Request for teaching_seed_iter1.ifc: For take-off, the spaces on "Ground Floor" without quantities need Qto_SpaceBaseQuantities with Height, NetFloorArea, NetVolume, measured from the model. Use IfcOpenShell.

First a look at what the model holds.

```python
import ifcopenshell
import ifcopenshell.util.element
import ifcopenshell.util.unit

model = ifcopenshell.open("teaching_seed_iter1.ifc")
print(model.schema)
for unit_type in ("LENGTHUNIT", "AREAUNIT", "VOLUMEUNIT"):
    print(unit_type, ifcopenshell.util.unit.calculate_unit_scale(model, unit_type))
storey = next(s for s in model.by_type("IfcBuildingStorey") if s.Name == "Ground Floor")
spaces = [e for e in ifcopenshell.util.element.get_decomposition(storey) if e.is_a("IfcSpace")]
for e in sorted(spaces, key=lambda e: e.id()):
    print(e.id(), e.is_a(), e.Name, list(ifcopenshell.util.element.get_psets(e, qtos_only=True)), sep=" | ")
```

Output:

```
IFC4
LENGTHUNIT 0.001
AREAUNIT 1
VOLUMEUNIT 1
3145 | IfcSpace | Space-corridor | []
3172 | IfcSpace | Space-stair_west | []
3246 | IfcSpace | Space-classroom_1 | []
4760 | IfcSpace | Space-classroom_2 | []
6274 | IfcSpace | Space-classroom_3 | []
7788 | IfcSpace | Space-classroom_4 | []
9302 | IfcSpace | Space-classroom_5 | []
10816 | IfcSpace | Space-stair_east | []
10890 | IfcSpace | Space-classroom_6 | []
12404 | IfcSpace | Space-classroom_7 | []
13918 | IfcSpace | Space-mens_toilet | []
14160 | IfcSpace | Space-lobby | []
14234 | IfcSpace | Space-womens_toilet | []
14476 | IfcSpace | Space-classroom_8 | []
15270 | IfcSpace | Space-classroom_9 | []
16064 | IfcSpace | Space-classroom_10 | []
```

```python
import ifcopenshell
import ifcopenshell.api.pset
import ifcopenshell.geom
import ifcopenshell.util.element
import ifcopenshell.util.shape
import ifcopenshell.util.unit

model = ifcopenshell.open("teaching_seed_iter1.ifc")
unit_scale = ifcopenshell.util.unit.calculate_unit_scale(model)
area_scale = ifcopenshell.util.unit.calculate_unit_scale(model, "AREAUNIT")
volume_scale = ifcopenshell.util.unit.calculate_unit_scale(model, "VOLUMEUNIT")
settings = ifcopenshell.geom.settings()

storey = next(s for s in model.by_type("IfcBuildingStorey") if s.Name == "Ground Floor")
spaces = [e for e in ifcopenshell.util.element.get_decomposition(storey) if e.is_a("IfcSpace")]

for e in sorted(spaces, key=lambda e: e.id()):
    if ifcopenshell.util.element.get_psets(e, qtos_only=True, should_inherit=False):
        continue
    # Geometry comes back in metres, in the element's own axes.
    shape = ifcopenshell.geom.create_shape(settings, e)
    values = {
        "Height": ifcopenshell.util.shape.get_z(shape.geometry) / unit_scale,
        "NetFloorArea": ifcopenshell.util.shape.get_footprint_area(shape.geometry) / area_scale,
        "NetVolume": ifcopenshell.util.shape.get_volume(shape.geometry) / volume_scale,
    }
    qto = ifcopenshell.api.pset.add_qto(model, product=e, name="Qto_SpaceBaseQuantities")
    ifcopenshell.api.pset.edit_qto(model, qto=qto, properties=values)
    print(e.id(), {k: round(v, 3) for k, v in values.items()})

model.write("teaching_seed_iter1_updated.ifc")
```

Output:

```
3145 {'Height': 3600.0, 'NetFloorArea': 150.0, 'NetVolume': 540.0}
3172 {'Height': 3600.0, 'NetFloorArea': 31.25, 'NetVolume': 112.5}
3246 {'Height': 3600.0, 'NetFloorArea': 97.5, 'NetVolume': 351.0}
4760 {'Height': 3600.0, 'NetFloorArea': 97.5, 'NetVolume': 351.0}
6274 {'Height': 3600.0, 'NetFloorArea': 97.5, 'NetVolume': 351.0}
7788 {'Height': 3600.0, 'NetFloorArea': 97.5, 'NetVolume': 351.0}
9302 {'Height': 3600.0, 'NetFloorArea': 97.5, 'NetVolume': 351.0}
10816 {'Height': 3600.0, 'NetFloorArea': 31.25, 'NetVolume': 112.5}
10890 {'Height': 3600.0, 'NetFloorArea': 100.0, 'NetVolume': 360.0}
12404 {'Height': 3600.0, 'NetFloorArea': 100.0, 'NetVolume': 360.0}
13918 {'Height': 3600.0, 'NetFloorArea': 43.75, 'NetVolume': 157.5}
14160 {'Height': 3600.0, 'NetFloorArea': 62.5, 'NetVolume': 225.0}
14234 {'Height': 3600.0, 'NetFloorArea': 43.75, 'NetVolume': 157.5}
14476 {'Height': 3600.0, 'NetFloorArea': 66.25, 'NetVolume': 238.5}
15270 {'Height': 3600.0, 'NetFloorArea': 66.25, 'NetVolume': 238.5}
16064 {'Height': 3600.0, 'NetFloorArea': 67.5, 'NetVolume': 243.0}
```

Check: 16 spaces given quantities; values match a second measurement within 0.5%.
